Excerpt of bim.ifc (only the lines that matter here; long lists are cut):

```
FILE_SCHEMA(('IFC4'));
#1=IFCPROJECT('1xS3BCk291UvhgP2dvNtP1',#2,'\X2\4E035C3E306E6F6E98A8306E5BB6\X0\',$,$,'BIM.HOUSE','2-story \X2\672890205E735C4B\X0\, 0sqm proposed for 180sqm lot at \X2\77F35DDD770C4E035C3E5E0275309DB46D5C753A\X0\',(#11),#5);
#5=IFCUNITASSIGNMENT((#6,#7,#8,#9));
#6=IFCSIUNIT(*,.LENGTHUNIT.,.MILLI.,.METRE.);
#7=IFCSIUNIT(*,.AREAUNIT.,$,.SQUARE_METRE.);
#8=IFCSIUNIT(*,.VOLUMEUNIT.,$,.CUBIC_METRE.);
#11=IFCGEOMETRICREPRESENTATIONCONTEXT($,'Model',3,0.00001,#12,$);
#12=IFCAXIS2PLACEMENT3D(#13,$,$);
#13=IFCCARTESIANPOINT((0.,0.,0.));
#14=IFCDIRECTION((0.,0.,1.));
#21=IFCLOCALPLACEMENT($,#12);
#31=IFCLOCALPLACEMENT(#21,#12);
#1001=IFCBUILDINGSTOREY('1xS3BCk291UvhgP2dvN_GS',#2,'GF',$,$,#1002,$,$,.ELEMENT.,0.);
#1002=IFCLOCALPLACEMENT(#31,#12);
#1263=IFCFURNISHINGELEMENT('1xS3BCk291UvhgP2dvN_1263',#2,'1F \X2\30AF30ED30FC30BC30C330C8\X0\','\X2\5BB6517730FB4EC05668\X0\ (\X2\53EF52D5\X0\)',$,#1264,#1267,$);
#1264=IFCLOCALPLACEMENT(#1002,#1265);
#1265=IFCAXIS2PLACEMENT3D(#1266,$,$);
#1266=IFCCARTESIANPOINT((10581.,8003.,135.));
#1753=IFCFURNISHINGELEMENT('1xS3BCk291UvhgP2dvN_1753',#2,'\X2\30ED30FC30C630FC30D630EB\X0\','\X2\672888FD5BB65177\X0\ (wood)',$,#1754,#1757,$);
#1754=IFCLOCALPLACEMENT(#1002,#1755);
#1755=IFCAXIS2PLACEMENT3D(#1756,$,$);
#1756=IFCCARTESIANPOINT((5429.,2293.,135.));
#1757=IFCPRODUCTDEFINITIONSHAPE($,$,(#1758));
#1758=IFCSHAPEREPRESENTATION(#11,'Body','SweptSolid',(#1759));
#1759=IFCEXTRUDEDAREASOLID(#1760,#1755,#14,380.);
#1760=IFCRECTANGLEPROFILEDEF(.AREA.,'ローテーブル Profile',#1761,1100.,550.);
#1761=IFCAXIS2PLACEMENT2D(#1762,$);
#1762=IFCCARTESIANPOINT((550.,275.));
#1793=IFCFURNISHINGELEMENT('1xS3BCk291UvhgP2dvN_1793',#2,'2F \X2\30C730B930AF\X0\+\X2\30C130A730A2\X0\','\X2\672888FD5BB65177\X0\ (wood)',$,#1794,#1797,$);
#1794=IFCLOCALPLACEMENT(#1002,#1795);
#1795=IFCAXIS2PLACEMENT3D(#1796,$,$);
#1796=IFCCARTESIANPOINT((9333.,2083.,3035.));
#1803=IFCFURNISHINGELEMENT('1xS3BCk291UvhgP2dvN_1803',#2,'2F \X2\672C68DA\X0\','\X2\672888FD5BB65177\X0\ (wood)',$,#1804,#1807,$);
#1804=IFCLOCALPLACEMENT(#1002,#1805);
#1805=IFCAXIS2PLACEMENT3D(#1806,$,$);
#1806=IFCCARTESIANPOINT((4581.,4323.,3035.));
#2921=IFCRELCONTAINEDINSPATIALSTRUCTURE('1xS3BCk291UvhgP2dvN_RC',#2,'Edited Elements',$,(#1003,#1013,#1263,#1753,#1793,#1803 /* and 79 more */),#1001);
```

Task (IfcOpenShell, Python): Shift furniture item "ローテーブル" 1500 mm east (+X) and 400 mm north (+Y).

```python
import ifcopenshell
import ifcopenshell.api.geometry
import ifcopenshell.util.placement
import ifcopenshell.util.unit

model = ifcopenshell.open("bim.ifc")
unit_scale = ifcopenshell.util.unit.calculate_unit_scale(model)

item = model.by_guid("1xS3BCk291UvhgP2dvN_1753")
matrix = ifcopenshell.util.placement.get_local_placement(item.ObjectPlacement)
matrix[0, 3] += 1.5 / unit_scale
matrix[1, 3] += 0.4 / unit_scale
ifcopenshell.api.geometry.edit_object_placement(model, product=item, matrix=matrix, is_si=False)

print(ifcopenshell.util.placement.get_local_placement(item.ObjectPlacement).round(3) + 0.0)

model.write("bim_rev.ifc")
```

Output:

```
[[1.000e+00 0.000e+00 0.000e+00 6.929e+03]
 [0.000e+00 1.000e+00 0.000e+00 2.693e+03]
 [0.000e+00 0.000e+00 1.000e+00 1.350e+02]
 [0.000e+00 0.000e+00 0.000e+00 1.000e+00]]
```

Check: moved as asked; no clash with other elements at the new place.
